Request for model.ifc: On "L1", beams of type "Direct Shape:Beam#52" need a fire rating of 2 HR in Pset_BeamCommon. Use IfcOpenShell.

First a look at what the model holds.

```python
import ifcopenshell
import ifcopenshell.util.element

model = ifcopenshell.open("model.ifc")
print(model.schema)
storey = next(s for s in model.by_type("IfcBuildingStorey") if s.Name == "L1")
beams = [e for e in ifcopenshell.util.element.get_decomposition(storey) if e.is_a("IfcBeam")]
seen = {}
for e in beams:
    element_type = ifcopenshell.util.element.get_type(e)
    key = (element_type.Name if element_type != e and element_type else None, ifcopenshell.util.element.get_pset(e, "Pset_BeamCommon", "FireRating"))
    seen[key] = seen.get(key, 0) + 1
for (name, value), count in sorted(seen.items(), key=str):
    print(count, "x", name, "|", value)
```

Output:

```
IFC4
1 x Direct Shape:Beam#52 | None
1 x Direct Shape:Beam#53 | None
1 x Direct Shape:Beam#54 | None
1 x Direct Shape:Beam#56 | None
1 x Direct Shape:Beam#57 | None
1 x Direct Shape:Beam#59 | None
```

```python
import ifcopenshell
import ifcopenshell.api.pset
import ifcopenshell.util.element

model = ifcopenshell.open("model.ifc")

storey = next(s for s in model.by_type("IfcBuildingStorey") if s.Name == "L1")
beams = [e for e in ifcopenshell.util.element.get_decomposition(storey) if e.is_a("IfcBeam")]

count = 0
for e in beams:
    element_type = ifcopenshell.util.element.get_type(e)
    if element_type in (None, e) or element_type.Name != "Direct Shape:Beam#52":
        continue
    # add_pset returns the element's existing set when there is one.
    pset = ifcopenshell.api.pset.add_pset(model, product=e, name="Pset_BeamCommon")
    ifcopenshell.api.pset.edit_pset(model, pset=pset, properties={"FireRating": "2 HR"})
    count += 1

print(count, "beams updated")

model.write("model_updated.ifc")
```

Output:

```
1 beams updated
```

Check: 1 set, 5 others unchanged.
